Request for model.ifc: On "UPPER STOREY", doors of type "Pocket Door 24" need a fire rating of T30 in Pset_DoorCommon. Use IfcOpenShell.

First a look at what the model holds.

```python
import ifcopenshell
import ifcopenshell.util.element

model = ifcopenshell.open("model.ifc")
print(model.schema)
storey = next(s for s in model.by_type("IfcBuildingStorey") if s.Name == "UPPER STOREY")
doors = [e for e in ifcopenshell.util.element.get_decomposition(storey) if e.is_a("IfcDoor")]
seen = {}
for e in doors:
    element_type = ifcopenshell.util.element.get_type(e)
    key = (element_type.Name if element_type != e and element_type else None, ifcopenshell.util.element.get_pset(e, "Pset_DoorCommon", "FireRating"))
    seen[key] = seen.get(key, 0) + 1
for (name, value), count in sorted(seen.items(), key=str):
    print(count, "x", name, "|", value)
```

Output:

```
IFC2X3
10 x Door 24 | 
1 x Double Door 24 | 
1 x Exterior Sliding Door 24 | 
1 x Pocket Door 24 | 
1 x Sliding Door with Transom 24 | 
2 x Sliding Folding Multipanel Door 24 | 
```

```python
import ifcopenshell
import ifcopenshell.api.pset
import ifcopenshell.util.element

model = ifcopenshell.open("model.ifc")

storey = next(s for s in model.by_type("IfcBuildingStorey") if s.Name == "UPPER STOREY")
doors = [e for e in ifcopenshell.util.element.get_decomposition(storey) if e.is_a("IfcDoor")]

count = 0
for e in doors:
    element_type = ifcopenshell.util.element.get_type(e)
    if element_type in (None, e) or element_type.Name != "Pocket Door 24":
        continue
    # add_pset returns the element's existing set when there is one.
    pset = ifcopenshell.api.pset.add_pset(model, product=e, name="Pset_DoorCommon")
    ifcopenshell.api.pset.edit_pset(model, pset=pset, properties={"FireRating": "T30"})
    count += 1

print(count, "doors updated")

model.write("model_rev.ifc")
```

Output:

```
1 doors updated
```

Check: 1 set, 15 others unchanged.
